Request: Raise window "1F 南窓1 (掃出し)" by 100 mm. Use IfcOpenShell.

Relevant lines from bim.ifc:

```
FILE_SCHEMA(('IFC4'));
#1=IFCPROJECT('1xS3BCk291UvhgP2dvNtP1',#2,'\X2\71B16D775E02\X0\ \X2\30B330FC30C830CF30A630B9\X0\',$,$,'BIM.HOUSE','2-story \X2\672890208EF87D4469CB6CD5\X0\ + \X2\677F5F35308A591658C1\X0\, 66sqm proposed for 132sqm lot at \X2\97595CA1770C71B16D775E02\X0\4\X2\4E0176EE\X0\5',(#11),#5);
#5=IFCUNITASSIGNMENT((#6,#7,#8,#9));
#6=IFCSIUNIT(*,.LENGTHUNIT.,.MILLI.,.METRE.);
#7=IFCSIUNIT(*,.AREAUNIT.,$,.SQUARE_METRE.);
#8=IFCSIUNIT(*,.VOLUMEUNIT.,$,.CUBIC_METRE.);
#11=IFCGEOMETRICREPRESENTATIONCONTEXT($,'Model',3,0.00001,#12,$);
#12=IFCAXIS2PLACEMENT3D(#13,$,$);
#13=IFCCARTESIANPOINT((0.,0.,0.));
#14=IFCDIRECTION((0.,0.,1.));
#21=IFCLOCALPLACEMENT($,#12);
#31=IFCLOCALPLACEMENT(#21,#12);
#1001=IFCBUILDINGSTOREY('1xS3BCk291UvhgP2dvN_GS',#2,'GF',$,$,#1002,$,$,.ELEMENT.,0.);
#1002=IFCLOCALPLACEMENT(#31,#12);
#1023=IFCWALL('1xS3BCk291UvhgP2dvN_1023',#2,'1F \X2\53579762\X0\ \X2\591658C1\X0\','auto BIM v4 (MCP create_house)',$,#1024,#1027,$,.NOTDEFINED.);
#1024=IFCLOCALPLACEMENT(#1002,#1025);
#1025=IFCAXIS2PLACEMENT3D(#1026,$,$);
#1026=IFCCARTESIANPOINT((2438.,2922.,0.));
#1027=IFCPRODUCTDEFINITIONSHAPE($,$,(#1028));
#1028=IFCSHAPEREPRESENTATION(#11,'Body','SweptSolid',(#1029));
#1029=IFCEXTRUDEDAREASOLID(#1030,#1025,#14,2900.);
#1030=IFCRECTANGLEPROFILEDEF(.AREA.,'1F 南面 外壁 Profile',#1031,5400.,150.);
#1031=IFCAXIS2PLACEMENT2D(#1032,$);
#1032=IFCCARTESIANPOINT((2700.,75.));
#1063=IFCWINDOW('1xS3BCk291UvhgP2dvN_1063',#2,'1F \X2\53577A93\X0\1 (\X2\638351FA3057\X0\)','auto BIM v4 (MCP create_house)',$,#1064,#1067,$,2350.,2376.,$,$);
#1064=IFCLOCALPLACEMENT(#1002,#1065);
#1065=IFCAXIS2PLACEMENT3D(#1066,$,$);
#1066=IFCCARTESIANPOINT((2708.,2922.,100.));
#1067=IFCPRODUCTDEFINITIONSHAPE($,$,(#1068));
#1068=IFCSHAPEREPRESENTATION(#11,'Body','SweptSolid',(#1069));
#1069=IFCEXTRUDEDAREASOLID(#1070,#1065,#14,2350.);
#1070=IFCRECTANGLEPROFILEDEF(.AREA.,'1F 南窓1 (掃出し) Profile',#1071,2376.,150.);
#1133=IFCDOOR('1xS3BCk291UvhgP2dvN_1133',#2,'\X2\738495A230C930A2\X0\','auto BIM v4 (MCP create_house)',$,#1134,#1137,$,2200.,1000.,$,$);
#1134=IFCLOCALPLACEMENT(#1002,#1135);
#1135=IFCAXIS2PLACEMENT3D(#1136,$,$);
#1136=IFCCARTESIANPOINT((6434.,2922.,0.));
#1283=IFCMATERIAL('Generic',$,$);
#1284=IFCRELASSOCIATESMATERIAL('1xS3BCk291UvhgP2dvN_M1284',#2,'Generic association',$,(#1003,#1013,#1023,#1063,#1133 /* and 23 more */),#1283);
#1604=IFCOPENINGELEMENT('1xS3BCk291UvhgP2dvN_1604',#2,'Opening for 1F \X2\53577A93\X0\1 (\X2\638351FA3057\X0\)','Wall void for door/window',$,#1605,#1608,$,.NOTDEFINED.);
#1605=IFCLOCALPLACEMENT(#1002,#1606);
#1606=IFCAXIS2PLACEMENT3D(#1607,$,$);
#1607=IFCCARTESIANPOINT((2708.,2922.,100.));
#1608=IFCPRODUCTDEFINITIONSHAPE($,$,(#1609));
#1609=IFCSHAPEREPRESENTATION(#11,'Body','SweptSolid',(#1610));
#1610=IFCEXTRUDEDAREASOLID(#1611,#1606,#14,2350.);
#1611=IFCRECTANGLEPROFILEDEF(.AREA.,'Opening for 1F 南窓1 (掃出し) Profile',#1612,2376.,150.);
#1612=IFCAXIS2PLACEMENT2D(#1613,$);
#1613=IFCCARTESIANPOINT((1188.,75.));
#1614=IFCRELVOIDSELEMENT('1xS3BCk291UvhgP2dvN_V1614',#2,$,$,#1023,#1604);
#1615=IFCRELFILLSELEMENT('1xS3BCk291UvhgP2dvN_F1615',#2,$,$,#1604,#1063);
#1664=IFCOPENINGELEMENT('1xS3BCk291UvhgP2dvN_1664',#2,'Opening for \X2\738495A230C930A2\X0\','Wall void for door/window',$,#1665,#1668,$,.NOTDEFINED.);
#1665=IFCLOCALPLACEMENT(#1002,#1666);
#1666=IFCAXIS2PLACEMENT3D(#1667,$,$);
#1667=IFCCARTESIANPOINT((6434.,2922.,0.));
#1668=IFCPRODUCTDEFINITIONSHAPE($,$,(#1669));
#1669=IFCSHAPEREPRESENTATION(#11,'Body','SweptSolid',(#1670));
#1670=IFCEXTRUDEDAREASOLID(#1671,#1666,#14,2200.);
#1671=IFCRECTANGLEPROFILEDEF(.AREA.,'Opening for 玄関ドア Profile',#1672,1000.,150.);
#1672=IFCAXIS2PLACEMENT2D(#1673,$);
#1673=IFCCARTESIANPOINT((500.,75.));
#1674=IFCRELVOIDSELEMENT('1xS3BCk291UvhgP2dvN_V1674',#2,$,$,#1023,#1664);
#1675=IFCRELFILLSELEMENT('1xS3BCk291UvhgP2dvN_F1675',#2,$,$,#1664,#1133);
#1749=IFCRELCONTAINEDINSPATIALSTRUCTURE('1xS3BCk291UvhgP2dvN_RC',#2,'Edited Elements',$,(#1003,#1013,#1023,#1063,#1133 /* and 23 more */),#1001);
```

```python
import numpy as np
import ifcopenshell
import ifcopenshell.api.geometry
import ifcopenshell.util.placement
import ifcopenshell.util.unit

model = ifcopenshell.open("bim.ifc")
unit_scale = ifcopenshell.util.unit.calculate_unit_scale(model)

window = model.by_id(1063)
opening = window.FillsVoids[0].RelatingOpeningElement
dz = 0.1 / unit_scale

shift = np.array([0.0, 0.0, dz])
# The window is not placed relative to its opening, so move both.
for product in (opening, window):
    matrix = ifcopenshell.util.placement.get_local_placement(product.ObjectPlacement)
    matrix[:3, 3] += shift
    ifcopenshell.api.geometry.edit_object_placement(model, product=product, matrix=matrix, is_si=False)

print(f"moved by {dz * unit_scale:+.3f} m")

model.write("bim_v2.ifc")
```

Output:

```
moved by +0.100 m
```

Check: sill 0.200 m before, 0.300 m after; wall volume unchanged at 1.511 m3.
